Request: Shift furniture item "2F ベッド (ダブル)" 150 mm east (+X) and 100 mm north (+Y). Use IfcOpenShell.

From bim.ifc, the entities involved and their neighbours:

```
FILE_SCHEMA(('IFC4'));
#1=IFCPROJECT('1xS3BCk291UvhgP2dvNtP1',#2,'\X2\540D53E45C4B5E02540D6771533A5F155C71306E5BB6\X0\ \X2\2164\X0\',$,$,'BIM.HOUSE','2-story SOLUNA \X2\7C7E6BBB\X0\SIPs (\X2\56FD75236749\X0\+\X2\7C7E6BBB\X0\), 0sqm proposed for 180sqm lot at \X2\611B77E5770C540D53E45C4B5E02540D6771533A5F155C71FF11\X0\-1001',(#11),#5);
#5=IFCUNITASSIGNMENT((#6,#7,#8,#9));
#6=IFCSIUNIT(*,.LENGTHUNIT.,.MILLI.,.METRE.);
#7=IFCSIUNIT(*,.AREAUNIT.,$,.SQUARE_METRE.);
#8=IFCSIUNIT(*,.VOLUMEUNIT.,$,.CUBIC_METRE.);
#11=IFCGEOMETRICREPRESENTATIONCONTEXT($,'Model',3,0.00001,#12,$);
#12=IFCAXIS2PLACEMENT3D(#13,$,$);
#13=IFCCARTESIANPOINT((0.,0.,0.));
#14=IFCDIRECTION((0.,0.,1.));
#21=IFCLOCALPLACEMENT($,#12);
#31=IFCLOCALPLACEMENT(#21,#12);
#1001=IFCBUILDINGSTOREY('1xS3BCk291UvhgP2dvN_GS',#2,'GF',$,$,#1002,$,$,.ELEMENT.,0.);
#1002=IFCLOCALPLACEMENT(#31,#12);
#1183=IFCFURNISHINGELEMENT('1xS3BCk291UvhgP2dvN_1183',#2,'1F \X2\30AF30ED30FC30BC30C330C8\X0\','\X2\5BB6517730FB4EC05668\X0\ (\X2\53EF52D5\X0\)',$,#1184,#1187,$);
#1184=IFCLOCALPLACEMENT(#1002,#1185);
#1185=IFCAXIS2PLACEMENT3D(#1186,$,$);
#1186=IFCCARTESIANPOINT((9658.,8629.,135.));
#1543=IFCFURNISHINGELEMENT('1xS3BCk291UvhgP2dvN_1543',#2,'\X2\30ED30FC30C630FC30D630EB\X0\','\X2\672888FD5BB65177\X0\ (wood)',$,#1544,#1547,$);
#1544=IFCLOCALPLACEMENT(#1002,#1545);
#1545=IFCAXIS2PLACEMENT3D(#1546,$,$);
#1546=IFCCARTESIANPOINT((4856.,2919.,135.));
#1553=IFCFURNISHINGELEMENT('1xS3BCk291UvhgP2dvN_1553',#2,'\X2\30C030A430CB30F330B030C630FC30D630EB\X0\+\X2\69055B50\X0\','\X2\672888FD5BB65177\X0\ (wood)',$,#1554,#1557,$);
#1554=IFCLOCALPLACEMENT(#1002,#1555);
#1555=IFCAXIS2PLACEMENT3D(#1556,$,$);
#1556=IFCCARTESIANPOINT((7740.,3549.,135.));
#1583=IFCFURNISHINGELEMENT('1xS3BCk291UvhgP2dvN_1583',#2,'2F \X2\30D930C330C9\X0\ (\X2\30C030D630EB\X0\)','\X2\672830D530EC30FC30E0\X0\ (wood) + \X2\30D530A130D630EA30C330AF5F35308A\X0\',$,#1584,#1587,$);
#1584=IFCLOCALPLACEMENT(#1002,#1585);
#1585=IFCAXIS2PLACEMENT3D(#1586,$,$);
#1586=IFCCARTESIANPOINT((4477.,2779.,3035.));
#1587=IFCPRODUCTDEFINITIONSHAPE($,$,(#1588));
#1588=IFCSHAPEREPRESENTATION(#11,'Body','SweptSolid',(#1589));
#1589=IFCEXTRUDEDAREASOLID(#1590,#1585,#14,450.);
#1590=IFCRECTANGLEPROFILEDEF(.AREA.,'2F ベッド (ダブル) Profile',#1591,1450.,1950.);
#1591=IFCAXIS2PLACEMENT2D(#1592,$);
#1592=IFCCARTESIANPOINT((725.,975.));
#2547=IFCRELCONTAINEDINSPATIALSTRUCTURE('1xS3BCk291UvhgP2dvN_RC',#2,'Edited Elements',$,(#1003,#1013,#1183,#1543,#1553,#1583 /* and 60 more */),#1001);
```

```python
import ifcopenshell
import ifcopenshell.api.geometry
import ifcopenshell.util.placement

model = ifcopenshell.open("bim.ifc")

item = model.by_guid("1xS3BCk291UvhgP2dvN_1583")
matrix = ifcopenshell.util.placement.get_local_placement(item.ObjectPlacement)
matrix[0, 3] += 150.0
matrix[1, 3] += 100.0
ifcopenshell.api.geometry.edit_object_placement(model, product=item, matrix=matrix, is_si=False)

print(ifcopenshell.util.placement.get_local_placement(item.ObjectPlacement).round(3) + 0.0)

model.write("bim_v2.ifc")
```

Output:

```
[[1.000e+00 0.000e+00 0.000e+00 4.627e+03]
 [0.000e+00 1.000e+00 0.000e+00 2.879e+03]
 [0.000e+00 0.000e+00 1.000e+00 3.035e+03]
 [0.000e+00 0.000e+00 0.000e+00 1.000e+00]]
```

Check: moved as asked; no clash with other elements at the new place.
